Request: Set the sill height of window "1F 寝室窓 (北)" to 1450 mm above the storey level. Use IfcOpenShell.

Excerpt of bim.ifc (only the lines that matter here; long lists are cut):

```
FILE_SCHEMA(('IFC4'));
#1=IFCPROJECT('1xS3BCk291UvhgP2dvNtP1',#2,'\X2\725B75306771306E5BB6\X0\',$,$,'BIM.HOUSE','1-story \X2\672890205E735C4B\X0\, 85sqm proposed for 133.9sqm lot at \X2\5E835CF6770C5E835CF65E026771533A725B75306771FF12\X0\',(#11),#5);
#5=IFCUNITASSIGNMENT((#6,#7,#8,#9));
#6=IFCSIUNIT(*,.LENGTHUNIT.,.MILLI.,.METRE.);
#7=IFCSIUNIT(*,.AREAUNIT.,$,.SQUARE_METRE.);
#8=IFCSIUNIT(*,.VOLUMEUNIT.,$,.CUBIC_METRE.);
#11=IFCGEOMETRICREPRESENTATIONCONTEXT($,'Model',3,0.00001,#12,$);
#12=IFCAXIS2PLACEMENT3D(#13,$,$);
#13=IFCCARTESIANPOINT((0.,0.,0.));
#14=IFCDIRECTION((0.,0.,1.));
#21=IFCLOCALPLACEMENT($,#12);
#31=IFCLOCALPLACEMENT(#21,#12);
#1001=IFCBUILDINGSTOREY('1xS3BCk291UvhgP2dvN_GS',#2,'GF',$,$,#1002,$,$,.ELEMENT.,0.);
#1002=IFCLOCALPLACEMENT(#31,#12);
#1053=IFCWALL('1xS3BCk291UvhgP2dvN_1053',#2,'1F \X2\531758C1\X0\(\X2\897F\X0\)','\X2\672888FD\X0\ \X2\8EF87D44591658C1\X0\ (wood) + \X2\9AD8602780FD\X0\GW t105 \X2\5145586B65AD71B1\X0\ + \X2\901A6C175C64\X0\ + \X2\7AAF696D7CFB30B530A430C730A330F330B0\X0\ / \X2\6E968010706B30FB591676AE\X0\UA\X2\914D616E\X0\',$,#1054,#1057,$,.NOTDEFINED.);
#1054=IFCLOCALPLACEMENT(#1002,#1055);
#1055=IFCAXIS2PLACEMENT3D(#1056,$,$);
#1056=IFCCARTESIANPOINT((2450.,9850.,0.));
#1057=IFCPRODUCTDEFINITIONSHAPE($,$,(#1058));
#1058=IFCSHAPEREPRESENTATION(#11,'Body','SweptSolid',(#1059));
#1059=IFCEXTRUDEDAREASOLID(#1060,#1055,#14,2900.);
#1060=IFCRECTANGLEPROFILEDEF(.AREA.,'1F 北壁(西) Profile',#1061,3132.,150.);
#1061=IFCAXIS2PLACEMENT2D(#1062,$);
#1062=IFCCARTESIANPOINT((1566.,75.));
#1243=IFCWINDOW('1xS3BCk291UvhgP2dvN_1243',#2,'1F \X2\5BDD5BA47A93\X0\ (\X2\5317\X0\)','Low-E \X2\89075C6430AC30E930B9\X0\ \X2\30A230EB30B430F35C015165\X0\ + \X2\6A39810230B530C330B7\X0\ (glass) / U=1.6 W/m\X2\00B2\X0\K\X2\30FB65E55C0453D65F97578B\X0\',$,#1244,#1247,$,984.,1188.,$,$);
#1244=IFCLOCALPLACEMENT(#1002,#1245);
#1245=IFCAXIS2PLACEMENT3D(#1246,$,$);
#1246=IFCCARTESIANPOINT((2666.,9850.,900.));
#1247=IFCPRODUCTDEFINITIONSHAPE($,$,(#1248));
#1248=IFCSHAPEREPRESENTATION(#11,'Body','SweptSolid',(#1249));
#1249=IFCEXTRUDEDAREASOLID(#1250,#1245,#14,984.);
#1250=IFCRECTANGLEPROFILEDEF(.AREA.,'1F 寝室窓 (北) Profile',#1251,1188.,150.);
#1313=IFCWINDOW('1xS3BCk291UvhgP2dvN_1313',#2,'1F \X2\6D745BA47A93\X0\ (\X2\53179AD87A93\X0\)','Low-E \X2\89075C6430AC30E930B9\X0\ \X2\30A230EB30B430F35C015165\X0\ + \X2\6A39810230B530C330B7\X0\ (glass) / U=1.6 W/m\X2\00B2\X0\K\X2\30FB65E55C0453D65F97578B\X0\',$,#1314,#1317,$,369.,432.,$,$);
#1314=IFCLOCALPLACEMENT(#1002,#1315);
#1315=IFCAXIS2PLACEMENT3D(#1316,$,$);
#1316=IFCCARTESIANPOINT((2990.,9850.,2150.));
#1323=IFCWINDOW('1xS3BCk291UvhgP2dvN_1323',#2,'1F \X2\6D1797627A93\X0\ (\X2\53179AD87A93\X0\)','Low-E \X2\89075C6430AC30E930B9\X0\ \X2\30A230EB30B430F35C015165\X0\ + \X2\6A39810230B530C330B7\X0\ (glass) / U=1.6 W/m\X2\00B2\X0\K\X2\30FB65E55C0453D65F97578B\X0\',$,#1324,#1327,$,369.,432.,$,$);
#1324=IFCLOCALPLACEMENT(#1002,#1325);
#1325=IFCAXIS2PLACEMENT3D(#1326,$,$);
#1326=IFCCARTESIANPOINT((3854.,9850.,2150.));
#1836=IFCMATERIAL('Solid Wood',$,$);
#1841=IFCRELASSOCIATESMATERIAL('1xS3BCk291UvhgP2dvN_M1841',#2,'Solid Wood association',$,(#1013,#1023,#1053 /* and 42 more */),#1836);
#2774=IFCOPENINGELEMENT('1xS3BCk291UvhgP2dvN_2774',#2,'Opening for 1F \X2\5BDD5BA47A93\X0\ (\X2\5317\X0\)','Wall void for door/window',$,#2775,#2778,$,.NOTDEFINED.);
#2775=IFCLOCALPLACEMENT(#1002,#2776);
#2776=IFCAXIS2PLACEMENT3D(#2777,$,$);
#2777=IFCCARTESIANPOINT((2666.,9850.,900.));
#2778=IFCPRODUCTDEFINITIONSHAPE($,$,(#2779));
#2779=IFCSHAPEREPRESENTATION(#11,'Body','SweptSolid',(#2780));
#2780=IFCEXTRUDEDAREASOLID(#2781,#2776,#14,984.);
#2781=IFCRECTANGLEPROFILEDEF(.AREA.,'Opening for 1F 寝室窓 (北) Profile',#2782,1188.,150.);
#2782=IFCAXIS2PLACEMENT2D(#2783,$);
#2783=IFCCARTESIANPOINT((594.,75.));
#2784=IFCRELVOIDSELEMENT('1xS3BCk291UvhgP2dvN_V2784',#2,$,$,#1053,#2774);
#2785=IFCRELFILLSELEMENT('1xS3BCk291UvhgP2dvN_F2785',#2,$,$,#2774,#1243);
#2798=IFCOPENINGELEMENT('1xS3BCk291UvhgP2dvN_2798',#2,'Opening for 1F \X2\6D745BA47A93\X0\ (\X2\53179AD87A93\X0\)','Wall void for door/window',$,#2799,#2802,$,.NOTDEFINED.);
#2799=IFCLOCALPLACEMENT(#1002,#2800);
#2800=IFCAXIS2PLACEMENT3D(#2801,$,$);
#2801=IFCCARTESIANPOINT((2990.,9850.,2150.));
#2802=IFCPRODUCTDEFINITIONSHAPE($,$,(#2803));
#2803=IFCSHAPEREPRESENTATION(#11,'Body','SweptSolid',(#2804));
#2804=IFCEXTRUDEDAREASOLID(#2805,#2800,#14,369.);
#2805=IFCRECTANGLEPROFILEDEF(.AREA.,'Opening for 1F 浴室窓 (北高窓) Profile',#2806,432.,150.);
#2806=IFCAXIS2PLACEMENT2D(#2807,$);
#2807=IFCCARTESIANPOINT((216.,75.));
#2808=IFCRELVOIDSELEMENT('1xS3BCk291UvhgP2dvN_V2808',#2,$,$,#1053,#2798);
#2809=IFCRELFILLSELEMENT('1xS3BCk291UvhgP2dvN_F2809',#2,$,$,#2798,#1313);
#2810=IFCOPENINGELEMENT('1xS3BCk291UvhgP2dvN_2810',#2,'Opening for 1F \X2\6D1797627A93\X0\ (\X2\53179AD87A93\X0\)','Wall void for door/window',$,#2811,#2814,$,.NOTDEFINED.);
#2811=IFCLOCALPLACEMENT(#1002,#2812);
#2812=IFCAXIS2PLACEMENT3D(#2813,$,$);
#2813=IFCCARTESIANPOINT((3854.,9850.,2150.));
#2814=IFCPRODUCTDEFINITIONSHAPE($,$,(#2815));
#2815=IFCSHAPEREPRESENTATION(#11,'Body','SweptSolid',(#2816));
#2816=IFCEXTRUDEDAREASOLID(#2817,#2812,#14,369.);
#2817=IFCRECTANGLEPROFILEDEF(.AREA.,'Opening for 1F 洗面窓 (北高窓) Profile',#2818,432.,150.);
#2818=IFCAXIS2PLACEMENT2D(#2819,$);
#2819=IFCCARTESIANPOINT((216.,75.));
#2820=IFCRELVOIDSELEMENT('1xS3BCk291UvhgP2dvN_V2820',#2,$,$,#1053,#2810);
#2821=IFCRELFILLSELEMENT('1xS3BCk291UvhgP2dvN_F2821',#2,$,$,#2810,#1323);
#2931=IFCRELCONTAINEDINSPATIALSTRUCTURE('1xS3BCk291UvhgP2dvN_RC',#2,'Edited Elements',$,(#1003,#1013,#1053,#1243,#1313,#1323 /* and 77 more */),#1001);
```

```python
import numpy as np
import ifcopenshell
import ifcopenshell.api.geometry
import ifcopenshell.geom
import ifcopenshell.util.element
import ifcopenshell.util.placement
import ifcopenshell.util.shape
import ifcopenshell.util.unit

model = ifcopenshell.open("bim.ifc")
unit_scale = ifcopenshell.util.unit.calculate_unit_scale(model)

window = model.by_id(1243)
opening = window.FillsVoids[0].RelatingOpeningElement
storey = ifcopenshell.util.element.get_container(window, ifc_class="IfcBuildingStorey")
level = ifcopenshell.util.placement.get_local_placement(storey.ObjectPlacement)[2, 3]

# The opening's origin need not be at the sill, so measure its lowest point.
shape = ifcopenshell.geom.create_shape(ifcopenshell.geom.settings(), opening)
bottom = ifcopenshell.util.shape.get_shape_bottom_elevation(shape, shape.geometry) / unit_scale
dz = level + 1.45 / unit_scale - bottom

shift = np.array([0.0, 0.0, dz])
# The window is not placed relative to its opening, so move both.
for product in (opening, window):
    matrix = ifcopenshell.util.placement.get_local_placement(product.ObjectPlacement)
    matrix[:3, 3] += shift
    ifcopenshell.api.geometry.edit_object_placement(model, product=product, matrix=matrix, is_si=False)

print(f"moved by {dz * unit_scale:+.3f} m")

model.write("bim_v2.ifc")
```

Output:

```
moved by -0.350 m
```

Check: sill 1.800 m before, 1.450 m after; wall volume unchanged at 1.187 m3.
